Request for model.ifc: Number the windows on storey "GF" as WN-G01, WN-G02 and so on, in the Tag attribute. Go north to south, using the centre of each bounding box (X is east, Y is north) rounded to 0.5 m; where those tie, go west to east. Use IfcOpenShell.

First a look at what the model holds.

```python
import ifcopenshell
import ifcopenshell.util.element
import ifcopenshell.util.placement

model = ifcopenshell.open("model.ifc")
print(model.schema)
storey = next(s for s in model.by_type("IfcBuildingStorey") if s.Name == "GF")
windows = [e for e in ifcopenshell.util.element.get_decomposition(storey) if e.is_a("IfcWindow")]
for e in sorted(windows, key=lambda e: e.id()):
    origin = ifcopenshell.util.placement.get_local_placement(e.ObjectPlacement)[:3, 3]
    print(e.id(), e.Tag, e.Name, origin.round(2) + 0.0, sep=" | ")
```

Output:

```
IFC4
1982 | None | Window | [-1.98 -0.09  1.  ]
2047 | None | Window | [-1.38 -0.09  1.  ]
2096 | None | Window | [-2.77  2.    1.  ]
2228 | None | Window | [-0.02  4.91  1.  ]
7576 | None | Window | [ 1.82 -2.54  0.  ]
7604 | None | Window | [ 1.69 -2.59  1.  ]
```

```python
import ifcopenshell
import ifcopenshell.geom
import ifcopenshell.util.element
import ifcopenshell.util.shape

model = ifcopenshell.open("model.ifc")
settings = ifcopenshell.geom.settings()
settings.set("use-world-coords", True)


def centre(element):
    shape = ifcopenshell.geom.create_shape(settings, element)
    return ifcopenshell.util.shape.get_bbox_centroid(shape.geometry)


storey = next(s for s in model.by_type("IfcBuildingStorey") if s.Name == "GF")
windows = [e for e in ifcopenshell.util.element.get_decomposition(storey) if e.is_a("IfcWindow")]

# Insertion points can sit at a corner or the storey origin, so sort by the geometry (in metres).
centres = {e: centre(e) for e in windows}
windows.sort(key=lambda e: (-round(centres[e][1] / 0.5), centres[e][0]))

for i, e in enumerate(windows, start=1):
    number = f"WN-G{i:02d}"
    e.Tag = number
    print(e.id(), number)

model.write("model_rev.ifc")
```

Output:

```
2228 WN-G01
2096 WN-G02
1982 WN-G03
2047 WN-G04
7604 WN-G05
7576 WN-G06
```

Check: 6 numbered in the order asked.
